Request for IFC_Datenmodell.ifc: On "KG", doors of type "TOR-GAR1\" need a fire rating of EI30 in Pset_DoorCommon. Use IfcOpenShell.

First a look at what the model holds.

```python
import ifcopenshell
import ifcopenshell.util.element

model = ifcopenshell.open("IFC_Datenmodell.ifc")
print(model.schema)
storey = next(s for s in model.by_type("IfcBuildingStorey") if s.Name == "KG")
doors = [e for e in ifcopenshell.util.element.get_decomposition(storey) if e.is_a("IfcDoor")]
seen = {}
for e in doors:
    element_type = ifcopenshell.util.element.get_type(e)
    key = (element_type.Name if element_type != e and element_type else None, ifcopenshell.util.element.get_pset(e, "Pset_DoorCommon", "FireRating"))
    seen[key] = seen.get(key, 0) + 1
for (name, value), count in sorted(seen.items(), key=str):
    print(count, "x", name, "|", value)
```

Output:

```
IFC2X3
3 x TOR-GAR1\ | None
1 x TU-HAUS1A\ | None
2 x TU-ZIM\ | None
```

```python
import ifcopenshell
import ifcopenshell.api.pset
import ifcopenshell.util.element

model = ifcopenshell.open("IFC_Datenmodell.ifc")

storey = next(s for s in model.by_type("IfcBuildingStorey") if s.Name == "KG")
doors = [e for e in ifcopenshell.util.element.get_decomposition(storey) if e.is_a("IfcDoor")]

count = 0
for e in doors:
    element_type = ifcopenshell.util.element.get_type(e)
    if element_type in (None, e) or element_type.Name != 'TOR-GAR1\\':
        continue
    # add_pset returns the element's existing set when there is one.
    pset = ifcopenshell.api.pset.add_pset(model, product=e, name="Pset_DoorCommon")
    ifcopenshell.api.pset.edit_pset(model, pset=pset, properties={"FireRating": "EI30"})
    count += 1

print(count, "doors updated")

model.write("IFC_Datenmodell_v2.ifc")
```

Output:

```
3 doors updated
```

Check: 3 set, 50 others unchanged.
